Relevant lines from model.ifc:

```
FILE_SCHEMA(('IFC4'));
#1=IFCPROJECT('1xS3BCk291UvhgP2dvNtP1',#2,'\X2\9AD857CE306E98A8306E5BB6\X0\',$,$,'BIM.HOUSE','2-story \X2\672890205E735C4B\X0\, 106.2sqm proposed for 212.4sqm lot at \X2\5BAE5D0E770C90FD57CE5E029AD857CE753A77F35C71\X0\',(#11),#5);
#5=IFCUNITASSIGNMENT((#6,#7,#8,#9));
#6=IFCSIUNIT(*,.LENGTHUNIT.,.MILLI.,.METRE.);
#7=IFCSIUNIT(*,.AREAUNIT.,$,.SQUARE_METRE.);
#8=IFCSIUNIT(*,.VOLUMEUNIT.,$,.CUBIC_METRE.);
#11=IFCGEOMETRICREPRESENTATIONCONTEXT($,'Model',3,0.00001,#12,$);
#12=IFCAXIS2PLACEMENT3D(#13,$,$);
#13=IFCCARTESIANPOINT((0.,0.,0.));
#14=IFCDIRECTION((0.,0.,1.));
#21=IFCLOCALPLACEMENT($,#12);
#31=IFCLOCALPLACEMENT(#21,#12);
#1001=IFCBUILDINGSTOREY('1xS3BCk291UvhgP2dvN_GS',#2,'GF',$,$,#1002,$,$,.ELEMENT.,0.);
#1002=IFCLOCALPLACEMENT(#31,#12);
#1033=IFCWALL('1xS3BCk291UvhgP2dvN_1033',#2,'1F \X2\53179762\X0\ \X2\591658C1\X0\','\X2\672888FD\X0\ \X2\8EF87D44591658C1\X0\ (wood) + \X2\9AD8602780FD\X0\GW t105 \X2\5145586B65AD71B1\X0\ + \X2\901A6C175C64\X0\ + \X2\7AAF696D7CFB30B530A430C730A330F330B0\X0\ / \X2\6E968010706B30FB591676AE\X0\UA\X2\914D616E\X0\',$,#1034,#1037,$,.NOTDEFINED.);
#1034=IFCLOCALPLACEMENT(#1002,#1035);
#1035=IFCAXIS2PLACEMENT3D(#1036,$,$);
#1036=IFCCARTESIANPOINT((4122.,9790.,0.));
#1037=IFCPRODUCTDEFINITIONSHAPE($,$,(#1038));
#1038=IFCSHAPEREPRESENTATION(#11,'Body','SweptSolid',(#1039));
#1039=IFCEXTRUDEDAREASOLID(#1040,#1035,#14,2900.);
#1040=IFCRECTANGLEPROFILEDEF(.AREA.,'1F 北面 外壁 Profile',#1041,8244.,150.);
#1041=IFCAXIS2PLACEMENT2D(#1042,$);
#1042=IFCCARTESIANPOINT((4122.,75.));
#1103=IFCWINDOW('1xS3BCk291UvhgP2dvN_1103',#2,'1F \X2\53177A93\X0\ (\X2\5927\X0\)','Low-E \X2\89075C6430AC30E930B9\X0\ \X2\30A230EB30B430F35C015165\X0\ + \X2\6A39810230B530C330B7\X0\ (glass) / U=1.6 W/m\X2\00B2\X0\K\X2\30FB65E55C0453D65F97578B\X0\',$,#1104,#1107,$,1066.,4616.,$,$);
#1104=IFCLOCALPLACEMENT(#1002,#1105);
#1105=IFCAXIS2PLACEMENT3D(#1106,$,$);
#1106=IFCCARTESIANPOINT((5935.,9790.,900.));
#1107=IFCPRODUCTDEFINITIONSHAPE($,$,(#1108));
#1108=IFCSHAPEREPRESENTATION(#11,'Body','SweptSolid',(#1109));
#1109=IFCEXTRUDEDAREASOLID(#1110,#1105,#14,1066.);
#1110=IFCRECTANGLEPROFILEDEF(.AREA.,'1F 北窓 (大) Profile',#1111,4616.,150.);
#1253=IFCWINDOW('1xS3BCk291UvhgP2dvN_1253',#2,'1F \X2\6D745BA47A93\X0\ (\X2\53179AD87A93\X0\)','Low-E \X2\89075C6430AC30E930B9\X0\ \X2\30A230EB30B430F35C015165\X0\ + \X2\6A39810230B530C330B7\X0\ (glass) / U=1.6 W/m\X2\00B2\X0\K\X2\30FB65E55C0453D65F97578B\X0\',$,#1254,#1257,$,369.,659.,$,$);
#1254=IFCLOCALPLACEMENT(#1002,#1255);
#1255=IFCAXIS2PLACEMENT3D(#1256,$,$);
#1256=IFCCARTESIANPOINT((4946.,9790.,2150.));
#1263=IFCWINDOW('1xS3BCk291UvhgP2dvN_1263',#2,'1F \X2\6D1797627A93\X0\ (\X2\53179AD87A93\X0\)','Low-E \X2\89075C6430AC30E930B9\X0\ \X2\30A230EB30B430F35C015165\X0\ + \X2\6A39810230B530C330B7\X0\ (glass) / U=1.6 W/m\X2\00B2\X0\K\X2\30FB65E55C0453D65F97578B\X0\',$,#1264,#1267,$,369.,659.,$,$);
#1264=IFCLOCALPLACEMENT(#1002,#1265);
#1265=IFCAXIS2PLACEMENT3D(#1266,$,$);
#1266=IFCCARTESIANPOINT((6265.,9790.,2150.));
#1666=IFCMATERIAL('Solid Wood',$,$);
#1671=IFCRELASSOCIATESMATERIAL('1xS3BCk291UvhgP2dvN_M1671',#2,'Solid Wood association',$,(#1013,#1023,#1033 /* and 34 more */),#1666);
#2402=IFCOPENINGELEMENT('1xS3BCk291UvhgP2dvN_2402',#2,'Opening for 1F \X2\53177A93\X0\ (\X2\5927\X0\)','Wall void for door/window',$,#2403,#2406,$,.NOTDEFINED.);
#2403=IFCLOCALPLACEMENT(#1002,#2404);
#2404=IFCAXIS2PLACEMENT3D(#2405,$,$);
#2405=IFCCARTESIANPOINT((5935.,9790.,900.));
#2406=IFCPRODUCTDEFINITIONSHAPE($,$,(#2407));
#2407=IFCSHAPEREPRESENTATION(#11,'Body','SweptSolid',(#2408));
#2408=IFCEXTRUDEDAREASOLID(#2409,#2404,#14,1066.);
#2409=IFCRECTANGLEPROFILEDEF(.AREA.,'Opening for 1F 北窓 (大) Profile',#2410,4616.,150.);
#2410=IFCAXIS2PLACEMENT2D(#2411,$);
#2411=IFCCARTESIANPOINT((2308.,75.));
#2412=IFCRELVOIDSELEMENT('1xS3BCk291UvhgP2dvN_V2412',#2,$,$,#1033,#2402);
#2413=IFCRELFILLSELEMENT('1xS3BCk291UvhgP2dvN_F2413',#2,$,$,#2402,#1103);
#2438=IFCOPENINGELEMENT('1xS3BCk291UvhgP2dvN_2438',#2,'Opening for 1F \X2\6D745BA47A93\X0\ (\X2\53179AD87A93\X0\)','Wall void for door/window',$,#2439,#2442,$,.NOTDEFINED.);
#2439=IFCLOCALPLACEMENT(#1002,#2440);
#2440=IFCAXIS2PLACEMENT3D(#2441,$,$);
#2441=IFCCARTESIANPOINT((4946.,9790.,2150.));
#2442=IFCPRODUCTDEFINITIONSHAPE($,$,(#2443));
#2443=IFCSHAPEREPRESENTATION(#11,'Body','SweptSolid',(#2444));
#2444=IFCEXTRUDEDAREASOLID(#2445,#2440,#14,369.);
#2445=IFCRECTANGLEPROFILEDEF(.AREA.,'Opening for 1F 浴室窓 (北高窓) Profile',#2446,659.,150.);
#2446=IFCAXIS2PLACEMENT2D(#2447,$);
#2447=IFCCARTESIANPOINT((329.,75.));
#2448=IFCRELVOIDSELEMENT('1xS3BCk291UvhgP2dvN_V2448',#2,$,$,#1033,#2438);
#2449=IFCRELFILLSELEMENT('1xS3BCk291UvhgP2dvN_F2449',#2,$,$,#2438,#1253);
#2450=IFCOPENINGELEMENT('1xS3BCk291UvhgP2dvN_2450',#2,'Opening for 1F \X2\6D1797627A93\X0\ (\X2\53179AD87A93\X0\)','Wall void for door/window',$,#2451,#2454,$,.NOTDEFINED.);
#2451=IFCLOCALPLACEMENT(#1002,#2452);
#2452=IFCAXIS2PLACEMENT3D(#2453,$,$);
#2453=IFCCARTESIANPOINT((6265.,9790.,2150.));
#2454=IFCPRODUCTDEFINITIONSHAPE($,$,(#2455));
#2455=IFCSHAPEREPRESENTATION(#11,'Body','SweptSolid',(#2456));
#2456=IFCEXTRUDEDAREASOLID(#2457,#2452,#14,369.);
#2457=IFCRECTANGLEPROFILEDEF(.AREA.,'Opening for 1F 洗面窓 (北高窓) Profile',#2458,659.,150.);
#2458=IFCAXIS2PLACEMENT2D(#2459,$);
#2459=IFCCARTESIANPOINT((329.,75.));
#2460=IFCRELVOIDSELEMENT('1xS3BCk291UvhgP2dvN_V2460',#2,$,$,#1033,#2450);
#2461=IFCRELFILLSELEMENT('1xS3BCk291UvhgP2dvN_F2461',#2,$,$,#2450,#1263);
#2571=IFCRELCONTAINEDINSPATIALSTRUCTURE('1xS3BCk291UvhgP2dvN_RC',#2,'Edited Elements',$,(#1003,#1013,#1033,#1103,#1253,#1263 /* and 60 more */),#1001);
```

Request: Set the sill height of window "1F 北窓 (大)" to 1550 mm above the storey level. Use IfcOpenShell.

```python
import numpy as np
import ifcopenshell
import ifcopenshell.api.geometry
import ifcopenshell.geom
import ifcopenshell.util.element
import ifcopenshell.util.placement
import ifcopenshell.util.shape
import ifcopenshell.util.unit

model = ifcopenshell.open("model.ifc")
unit_scale = ifcopenshell.util.unit.calculate_unit_scale(model)

window = model.by_id(1103)
opening = window.FillsVoids[0].RelatingOpeningElement
storey = ifcopenshell.util.element.get_container(window, ifc_class="IfcBuildingStorey")
level = ifcopenshell.util.placement.get_local_placement(storey.ObjectPlacement)[2, 3]

# The opening's origin need not be at the sill, so measure its lowest point.
shape = ifcopenshell.geom.create_shape(ifcopenshell.geom.settings(), opening)
bottom = ifcopenshell.util.shape.get_shape_bottom_elevation(shape, shape.geometry) / unit_scale
dz = level + 1.55 / unit_scale - bottom

shift = np.array([0.0, 0.0, dz])
# The window is not placed relative to its opening, so move both.
for product in (opening, window):
    matrix = ifcopenshell.util.placement.get_local_placement(product.ObjectPlacement)
    matrix[:3, 3] += shift
    ifcopenshell.api.geometry.edit_object_placement(model, product=product, matrix=matrix, is_si=False)

print(f"moved by {dz * unit_scale:+.3f} m")

model.write("model_v2.ifc")
```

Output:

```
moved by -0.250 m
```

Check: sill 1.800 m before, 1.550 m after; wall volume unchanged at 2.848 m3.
